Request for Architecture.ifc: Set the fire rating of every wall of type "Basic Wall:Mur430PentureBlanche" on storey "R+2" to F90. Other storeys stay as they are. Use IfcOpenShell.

First a look at what the model holds.

```python
import ifcopenshell
import ifcopenshell.util.element

model = ifcopenshell.open("Architecture.ifc")
print(model.schema)
storey = next(s for s in model.by_type("IfcBuildingStorey") if s.Name == "R+2")
walls = [e for e in ifcopenshell.util.element.get_decomposition(storey) if e.is_a("IfcWall")]
seen = {}
for e in walls:
    element_type = ifcopenshell.util.element.get_type(e)
    key = (element_type.Name if element_type != e and element_type else None, ifcopenshell.util.element.get_pset(e, "Pset_WallCommon", "FireRating"))
    seen[key] = seen.get(key, 0) + 1
for (name, value), count in sorted(seen.items(), key=str):
    print(count, "x", name, "|", value)
```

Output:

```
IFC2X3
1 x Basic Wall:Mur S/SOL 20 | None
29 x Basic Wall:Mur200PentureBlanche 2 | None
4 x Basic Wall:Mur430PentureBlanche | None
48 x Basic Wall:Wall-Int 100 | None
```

```python
import ifcopenshell
import ifcopenshell.api.pset
import ifcopenshell.util.element

model = ifcopenshell.open("Architecture.ifc")

storey = next(s for s in model.by_type("IfcBuildingStorey") if s.Name == "R+2")
walls = [e for e in ifcopenshell.util.element.get_decomposition(storey) if e.is_a("IfcWall")]

count = 0
for e in walls:
    element_type = ifcopenshell.util.element.get_type(e)
    if element_type in (None, e) or element_type.Name != "Basic Wall:Mur430PentureBlanche":
        continue
    # add_pset returns the element's existing set when there is one.
    pset = ifcopenshell.api.pset.add_pset(model, product=e, name="Pset_WallCommon")
    ifcopenshell.api.pset.edit_pset(model, pset=pset, properties={"FireRating": "F90"})
    count += 1

print(count, "walls updated")

model.write("Architecture_v2.ifc")
```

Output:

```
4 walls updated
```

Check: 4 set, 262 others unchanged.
